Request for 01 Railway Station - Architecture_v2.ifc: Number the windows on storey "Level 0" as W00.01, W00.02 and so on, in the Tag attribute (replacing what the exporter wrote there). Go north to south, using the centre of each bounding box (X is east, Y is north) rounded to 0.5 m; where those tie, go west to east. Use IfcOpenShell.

First a look at what the model holds.

```python
import ifcopenshell
import ifcopenshell.util.element
import ifcopenshell.util.placement

model = ifcopenshell.open("01 Railway Station - Architecture_v2.ifc")
print(model.schema)
storey = next(s for s in model.by_type("IfcBuildingStorey") if s.Name == "Level 0")
windows = [e for e in ifcopenshell.util.element.get_decomposition(storey) if e.is_a("IfcWindow")]
for e in sorted(windows, key=lambda e: e.id()):
    origin = ifcopenshell.util.placement.get_local_placement(e.ObjectPlacement)[:3, 3]
    print(e.id(), e.Tag, e.Name, origin.round(2) + 0.0, sep=" | ")
```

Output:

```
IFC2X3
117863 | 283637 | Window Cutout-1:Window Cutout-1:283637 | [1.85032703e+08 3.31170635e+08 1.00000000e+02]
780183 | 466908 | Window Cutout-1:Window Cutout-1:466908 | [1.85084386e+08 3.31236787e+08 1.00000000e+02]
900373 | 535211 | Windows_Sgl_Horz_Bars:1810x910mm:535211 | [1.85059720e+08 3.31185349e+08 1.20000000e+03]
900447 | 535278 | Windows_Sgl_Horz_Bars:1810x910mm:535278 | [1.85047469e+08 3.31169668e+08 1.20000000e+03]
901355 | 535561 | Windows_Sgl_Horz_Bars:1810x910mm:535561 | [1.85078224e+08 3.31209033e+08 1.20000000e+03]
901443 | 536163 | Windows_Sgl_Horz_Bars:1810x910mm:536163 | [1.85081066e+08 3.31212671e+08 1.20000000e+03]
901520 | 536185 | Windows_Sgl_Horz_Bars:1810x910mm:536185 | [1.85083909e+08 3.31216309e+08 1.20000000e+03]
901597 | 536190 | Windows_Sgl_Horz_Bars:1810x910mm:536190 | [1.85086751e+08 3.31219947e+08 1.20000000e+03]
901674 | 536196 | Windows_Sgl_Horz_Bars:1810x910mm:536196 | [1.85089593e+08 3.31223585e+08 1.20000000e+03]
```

```python
import ifcopenshell
import ifcopenshell.geom
import ifcopenshell.util.element
import ifcopenshell.util.shape

model = ifcopenshell.open("01 Railway Station - Architecture_v2.ifc")
settings = ifcopenshell.geom.settings()
settings.set("use-world-coords", True)


def centre(element):
    shape = ifcopenshell.geom.create_shape(settings, element)
    return ifcopenshell.util.shape.get_bbox_centroid(shape.geometry)


storey = next(s for s in model.by_type("IfcBuildingStorey") if s.Name == "Level 0")
windows = [e for e in ifcopenshell.util.element.get_decomposition(storey) if e.is_a("IfcWindow")]

# Insertion points can sit at a corner or the storey origin, so sort by the geometry (in metres).
centres = {e: centre(e) for e in windows}
windows.sort(key=lambda e: (-round(centres[e][1] / 0.5), centres[e][0]))

for i, e in enumerate(windows, start=1):
    number = f"W00.{i:02d}"
    e.Tag = number
    print(e.id(), number)

model.write("01 Railway Station - Architecture_v2-out.ifc")
```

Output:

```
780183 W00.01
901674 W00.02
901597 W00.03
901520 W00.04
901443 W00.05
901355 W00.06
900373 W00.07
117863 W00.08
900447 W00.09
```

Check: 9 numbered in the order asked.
